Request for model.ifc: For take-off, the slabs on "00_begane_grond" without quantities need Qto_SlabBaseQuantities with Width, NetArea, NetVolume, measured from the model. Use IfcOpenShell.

First a look at what the model holds.

```python
import ifcopenshell
import ifcopenshell.util.element
import ifcopenshell.util.unit

model = ifcopenshell.open("model.ifc")
print(model.schema)
for unit_type in ("LENGTHUNIT", "AREAUNIT", "VOLUMEUNIT"):
    print(unit_type, ifcopenshell.util.unit.calculate_unit_scale(model, unit_type))
storey = next(s for s in model.by_type("IfcBuildingStorey") if s.Name == "00_begane_grond")
slabs = [e for e in ifcopenshell.util.element.get_decomposition(storey) if e.is_a("IfcSlab")]
for e in sorted(slabs, key=lambda e: e.id()):
    print(e.id(), e.is_a(), e.Name, list(ifcopenshell.util.element.get_psets(e, qtos_only=True)), sep=" | ")
```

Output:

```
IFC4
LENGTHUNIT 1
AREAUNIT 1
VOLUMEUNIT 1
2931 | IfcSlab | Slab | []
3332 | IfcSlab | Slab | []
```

```python
import ifcopenshell
import ifcopenshell.api.pset
import ifcopenshell.geom
import ifcopenshell.util.element
import ifcopenshell.util.shape
import ifcopenshell.util.unit

model = ifcopenshell.open("model.ifc")
unit_scale = ifcopenshell.util.unit.calculate_unit_scale(model)
area_scale = ifcopenshell.util.unit.calculate_unit_scale(model, "AREAUNIT")
volume_scale = ifcopenshell.util.unit.calculate_unit_scale(model, "VOLUMEUNIT")
settings = ifcopenshell.geom.settings()

storey = next(s for s in model.by_type("IfcBuildingStorey") if s.Name == "00_begane_grond")
slabs = [e for e in ifcopenshell.util.element.get_decomposition(storey) if e.is_a("IfcSlab")]

for e in sorted(slabs, key=lambda e: e.id()):
    if ifcopenshell.util.element.get_psets(e, qtos_only=True, should_inherit=False):
        continue
    # Geometry comes back in metres, in the element's own axes.
    shape = ifcopenshell.geom.create_shape(settings, e)
    values = {
        "Width": ifcopenshell.util.shape.get_z(shape.geometry) / unit_scale,
        "NetArea": ifcopenshell.util.shape.get_footprint_area(shape.geometry) / area_scale,
        "NetVolume": ifcopenshell.util.shape.get_volume(shape.geometry) / volume_scale,
    }
    qto = ifcopenshell.api.pset.add_qto(model, product=e, name="Qto_SlabBaseQuantities")
    ifcopenshell.api.pset.edit_qto(model, qto=qto, properties=values)
    print(e.id(), {k: round(v, 3) for k, v in values.items()})

model.write("model_v2.ifc")
```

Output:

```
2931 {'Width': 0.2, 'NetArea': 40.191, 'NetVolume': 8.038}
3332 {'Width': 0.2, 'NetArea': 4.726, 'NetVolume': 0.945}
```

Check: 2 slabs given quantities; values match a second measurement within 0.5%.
